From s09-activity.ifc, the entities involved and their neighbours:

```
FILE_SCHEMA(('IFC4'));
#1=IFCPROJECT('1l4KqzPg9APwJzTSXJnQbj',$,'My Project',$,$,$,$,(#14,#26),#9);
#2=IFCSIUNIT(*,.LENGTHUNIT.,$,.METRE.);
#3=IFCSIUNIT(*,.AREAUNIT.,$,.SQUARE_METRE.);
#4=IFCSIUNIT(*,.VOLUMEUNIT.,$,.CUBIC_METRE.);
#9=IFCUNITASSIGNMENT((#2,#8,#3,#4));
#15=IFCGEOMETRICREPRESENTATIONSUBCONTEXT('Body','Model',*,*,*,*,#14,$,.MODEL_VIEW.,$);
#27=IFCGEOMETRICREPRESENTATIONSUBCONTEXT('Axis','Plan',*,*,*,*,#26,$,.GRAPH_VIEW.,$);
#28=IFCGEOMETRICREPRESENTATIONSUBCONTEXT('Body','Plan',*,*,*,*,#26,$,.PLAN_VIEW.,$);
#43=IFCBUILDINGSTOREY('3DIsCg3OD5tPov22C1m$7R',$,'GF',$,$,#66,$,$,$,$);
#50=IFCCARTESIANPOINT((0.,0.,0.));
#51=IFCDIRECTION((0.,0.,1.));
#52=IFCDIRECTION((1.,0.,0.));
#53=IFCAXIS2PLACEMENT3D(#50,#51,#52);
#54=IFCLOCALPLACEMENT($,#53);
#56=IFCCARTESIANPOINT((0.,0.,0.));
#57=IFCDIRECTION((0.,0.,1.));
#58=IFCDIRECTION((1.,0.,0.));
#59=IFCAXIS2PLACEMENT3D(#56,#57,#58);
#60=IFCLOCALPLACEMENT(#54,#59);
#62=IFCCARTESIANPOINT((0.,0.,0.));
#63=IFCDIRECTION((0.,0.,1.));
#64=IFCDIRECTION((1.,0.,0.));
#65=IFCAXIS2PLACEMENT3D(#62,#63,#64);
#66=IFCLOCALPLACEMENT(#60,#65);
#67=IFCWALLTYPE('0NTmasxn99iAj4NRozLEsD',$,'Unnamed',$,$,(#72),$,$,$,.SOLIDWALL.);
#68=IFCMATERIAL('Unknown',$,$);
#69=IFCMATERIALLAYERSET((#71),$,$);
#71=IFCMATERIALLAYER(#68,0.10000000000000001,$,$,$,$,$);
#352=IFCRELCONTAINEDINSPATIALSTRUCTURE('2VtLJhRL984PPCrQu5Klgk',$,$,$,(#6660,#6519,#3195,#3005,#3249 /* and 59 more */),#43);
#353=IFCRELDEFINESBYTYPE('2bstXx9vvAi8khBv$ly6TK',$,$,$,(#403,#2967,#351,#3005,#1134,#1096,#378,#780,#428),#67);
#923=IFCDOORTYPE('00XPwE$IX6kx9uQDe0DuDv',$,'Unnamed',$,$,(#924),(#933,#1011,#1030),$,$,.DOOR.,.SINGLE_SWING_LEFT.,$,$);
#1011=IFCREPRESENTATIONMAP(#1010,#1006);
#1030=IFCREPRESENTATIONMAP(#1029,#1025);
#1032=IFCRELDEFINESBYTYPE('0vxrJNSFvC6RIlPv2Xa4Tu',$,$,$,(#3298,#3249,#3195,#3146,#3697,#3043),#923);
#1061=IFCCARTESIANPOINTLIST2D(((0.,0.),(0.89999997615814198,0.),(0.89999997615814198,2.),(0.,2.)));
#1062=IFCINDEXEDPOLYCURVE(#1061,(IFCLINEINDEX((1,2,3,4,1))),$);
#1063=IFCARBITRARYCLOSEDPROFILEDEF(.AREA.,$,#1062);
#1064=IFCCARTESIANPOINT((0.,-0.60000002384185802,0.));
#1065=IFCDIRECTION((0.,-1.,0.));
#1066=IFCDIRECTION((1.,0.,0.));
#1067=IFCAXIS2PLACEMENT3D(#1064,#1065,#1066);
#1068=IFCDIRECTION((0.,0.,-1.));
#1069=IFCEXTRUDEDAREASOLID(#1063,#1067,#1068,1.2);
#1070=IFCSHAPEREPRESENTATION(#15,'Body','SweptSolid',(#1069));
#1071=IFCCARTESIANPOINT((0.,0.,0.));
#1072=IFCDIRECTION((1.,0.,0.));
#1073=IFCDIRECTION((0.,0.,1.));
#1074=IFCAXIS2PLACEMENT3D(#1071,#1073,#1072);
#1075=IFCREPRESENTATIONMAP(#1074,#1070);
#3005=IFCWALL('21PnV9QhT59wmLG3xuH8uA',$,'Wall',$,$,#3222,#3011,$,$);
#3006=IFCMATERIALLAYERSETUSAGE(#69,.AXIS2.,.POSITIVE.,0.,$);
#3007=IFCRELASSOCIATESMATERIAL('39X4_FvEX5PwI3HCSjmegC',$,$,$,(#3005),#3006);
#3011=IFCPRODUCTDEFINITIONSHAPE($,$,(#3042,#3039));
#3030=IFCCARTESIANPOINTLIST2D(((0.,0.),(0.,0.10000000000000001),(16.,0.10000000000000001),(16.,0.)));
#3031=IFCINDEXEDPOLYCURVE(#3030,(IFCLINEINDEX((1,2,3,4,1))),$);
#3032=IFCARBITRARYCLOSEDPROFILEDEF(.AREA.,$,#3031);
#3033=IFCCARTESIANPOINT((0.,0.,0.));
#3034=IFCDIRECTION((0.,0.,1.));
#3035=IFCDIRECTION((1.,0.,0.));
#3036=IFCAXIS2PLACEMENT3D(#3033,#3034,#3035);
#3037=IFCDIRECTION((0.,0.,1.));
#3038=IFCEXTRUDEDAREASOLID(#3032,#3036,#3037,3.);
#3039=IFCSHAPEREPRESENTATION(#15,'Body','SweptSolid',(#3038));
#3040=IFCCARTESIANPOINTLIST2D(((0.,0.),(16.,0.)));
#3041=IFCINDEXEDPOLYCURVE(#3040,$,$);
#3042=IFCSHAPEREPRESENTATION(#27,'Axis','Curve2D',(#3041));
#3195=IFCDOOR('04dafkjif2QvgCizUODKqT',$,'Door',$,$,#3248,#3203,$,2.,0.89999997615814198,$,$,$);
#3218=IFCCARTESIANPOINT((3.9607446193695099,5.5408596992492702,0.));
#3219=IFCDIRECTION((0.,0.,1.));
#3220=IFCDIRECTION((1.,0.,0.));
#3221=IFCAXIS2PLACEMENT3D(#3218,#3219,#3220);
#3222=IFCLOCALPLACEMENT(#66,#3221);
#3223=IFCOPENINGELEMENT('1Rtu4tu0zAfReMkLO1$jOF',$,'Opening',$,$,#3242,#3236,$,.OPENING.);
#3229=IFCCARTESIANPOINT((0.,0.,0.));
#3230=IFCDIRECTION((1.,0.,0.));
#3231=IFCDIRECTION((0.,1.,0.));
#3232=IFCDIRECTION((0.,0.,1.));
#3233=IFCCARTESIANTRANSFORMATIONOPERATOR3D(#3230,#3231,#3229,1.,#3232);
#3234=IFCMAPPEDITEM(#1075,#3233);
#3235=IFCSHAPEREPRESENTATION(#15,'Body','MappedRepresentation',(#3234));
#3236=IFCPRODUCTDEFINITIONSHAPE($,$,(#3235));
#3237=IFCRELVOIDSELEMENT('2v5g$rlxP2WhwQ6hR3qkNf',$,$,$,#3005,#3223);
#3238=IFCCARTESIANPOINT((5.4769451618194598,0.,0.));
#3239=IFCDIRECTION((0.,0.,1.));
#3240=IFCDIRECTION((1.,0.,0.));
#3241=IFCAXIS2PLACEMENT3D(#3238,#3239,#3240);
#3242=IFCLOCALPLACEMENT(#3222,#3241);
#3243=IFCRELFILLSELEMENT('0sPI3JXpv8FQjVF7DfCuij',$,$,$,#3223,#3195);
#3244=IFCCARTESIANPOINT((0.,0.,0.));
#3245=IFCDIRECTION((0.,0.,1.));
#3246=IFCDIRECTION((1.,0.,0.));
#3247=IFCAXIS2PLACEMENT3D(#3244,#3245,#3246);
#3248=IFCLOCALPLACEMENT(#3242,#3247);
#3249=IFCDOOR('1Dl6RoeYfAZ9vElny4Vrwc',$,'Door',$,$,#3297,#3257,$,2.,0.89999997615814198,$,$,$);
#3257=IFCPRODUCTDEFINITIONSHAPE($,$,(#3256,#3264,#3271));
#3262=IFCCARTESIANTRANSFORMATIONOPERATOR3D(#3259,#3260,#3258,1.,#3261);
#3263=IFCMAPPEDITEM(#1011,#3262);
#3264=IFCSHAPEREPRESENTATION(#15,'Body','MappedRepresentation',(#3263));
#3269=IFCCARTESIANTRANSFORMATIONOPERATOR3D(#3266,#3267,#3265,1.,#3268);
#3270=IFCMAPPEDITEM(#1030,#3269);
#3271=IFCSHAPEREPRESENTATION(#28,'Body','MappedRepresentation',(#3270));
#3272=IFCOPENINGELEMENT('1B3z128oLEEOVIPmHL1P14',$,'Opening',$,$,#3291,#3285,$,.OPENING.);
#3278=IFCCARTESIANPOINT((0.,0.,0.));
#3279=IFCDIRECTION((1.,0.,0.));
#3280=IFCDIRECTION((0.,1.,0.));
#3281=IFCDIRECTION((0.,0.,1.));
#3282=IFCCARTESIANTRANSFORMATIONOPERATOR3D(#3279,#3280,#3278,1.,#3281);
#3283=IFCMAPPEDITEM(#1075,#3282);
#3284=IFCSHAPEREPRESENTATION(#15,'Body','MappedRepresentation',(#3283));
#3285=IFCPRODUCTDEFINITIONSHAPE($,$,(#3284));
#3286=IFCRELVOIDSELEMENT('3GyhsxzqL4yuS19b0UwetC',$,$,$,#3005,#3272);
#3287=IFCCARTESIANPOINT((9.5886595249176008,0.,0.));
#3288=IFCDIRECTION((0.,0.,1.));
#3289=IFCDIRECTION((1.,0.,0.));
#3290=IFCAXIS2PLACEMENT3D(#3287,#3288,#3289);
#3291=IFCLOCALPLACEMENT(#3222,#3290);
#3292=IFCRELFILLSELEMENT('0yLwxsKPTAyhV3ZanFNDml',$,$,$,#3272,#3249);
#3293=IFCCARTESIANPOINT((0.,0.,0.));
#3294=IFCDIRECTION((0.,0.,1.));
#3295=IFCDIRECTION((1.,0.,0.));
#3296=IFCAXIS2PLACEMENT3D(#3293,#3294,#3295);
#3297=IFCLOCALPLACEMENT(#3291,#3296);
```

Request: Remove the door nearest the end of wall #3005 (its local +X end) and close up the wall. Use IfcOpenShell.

```python
import ifcopenshell
import ifcopenshell.api.feature
import ifcopenshell.api.root
import ifcopenshell.geom
import ifcopenshell.util.shape

model = ifcopenshell.open("s09-activity.ifc")
settings = ifcopenshell.geom.settings()


def volume(element):
    """Net volume in cubic metres, openings subtracted."""
    shape = ifcopenshell.geom.create_shape(settings, element)
    return ifcopenshell.util.shape.get_volume(shape.geometry)


door = model.by_guid("1Dl6RoeYfAZ9vElny4Vrwc")
opening = door.FillsVoids[0].RelatingOpeningElement
wall = opening.VoidsElements[0].RelatingBuildingElement
before = volume(wall)

ifcopenshell.api.root.remove_product(model, product=door)
ifcopenshell.api.feature.remove_feature(model, feature=opening)

after = volume(wall)

print(f"wall volume {before:.3f} -> {after:.3f} m3")

model.write("s09-activity_v2.ifc")
```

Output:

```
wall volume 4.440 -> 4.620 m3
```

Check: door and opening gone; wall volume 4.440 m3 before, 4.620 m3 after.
